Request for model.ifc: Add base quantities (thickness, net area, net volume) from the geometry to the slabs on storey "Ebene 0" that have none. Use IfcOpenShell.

First a look at what the model holds.

```python
import ifcopenshell
import ifcopenshell.util.element
import ifcopenshell.util.unit

model = ifcopenshell.open("model.ifc")
print(model.schema)
for unit_type in ("LENGTHUNIT", "AREAUNIT", "VOLUMEUNIT"):
    print(unit_type, ifcopenshell.util.unit.calculate_unit_scale(model, unit_type))
storey = next(s for s in model.by_type("IfcBuildingStorey") if s.Name == "Ebene 0")
slabs = [e for e in ifcopenshell.util.element.get_decomposition(storey) if e.is_a("IfcSlab")]
for e in sorted(slabs, key=lambda e: e.id()):
    print(e.id(), e.is_a(), e.Name, list(ifcopenshell.util.element.get_psets(e, qtos_only=True)), sep=" | ")
```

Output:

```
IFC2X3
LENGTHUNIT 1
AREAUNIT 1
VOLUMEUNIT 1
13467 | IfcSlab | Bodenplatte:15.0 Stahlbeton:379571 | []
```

```python
import ifcopenshell
import ifcopenshell.api.pset
import ifcopenshell.geom
import ifcopenshell.util.element
import ifcopenshell.util.shape
import ifcopenshell.util.unit

model = ifcopenshell.open("model.ifc")
unit_scale = ifcopenshell.util.unit.calculate_unit_scale(model)
area_scale = ifcopenshell.util.unit.calculate_unit_scale(model, "AREAUNIT")
volume_scale = ifcopenshell.util.unit.calculate_unit_scale(model, "VOLUMEUNIT")
settings = ifcopenshell.geom.settings()

storey = next(s for s in model.by_type("IfcBuildingStorey") if s.Name == "Ebene 0")
slabs = [e for e in ifcopenshell.util.element.get_decomposition(storey) if e.is_a("IfcSlab")]

for e in sorted(slabs, key=lambda e: e.id()):
    if ifcopenshell.util.element.get_psets(e, qtos_only=True, should_inherit=False):
        continue
    # Geometry comes back in metres, in the element's own axes.
    shape = ifcopenshell.geom.create_shape(settings, e)
    values = {
        "Width": ifcopenshell.util.shape.get_z(shape.geometry) / unit_scale,
        "NetArea": ifcopenshell.util.shape.get_footprint_area(shape.geometry) / area_scale,
        "NetVolume": ifcopenshell.util.shape.get_volume(shape.geometry) / volume_scale,
    }
    qto = ifcopenshell.api.pset.add_qto(model, product=e, name="BaseQuantities")
    ifcopenshell.api.pset.edit_qto(model, qto=qto, properties=values)
    print(e.id(), {k: round(v, 3) for k, v in values.items()})

model.write("model_v2.ifc")
```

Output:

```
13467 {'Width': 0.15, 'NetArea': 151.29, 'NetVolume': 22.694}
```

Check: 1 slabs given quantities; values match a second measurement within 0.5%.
